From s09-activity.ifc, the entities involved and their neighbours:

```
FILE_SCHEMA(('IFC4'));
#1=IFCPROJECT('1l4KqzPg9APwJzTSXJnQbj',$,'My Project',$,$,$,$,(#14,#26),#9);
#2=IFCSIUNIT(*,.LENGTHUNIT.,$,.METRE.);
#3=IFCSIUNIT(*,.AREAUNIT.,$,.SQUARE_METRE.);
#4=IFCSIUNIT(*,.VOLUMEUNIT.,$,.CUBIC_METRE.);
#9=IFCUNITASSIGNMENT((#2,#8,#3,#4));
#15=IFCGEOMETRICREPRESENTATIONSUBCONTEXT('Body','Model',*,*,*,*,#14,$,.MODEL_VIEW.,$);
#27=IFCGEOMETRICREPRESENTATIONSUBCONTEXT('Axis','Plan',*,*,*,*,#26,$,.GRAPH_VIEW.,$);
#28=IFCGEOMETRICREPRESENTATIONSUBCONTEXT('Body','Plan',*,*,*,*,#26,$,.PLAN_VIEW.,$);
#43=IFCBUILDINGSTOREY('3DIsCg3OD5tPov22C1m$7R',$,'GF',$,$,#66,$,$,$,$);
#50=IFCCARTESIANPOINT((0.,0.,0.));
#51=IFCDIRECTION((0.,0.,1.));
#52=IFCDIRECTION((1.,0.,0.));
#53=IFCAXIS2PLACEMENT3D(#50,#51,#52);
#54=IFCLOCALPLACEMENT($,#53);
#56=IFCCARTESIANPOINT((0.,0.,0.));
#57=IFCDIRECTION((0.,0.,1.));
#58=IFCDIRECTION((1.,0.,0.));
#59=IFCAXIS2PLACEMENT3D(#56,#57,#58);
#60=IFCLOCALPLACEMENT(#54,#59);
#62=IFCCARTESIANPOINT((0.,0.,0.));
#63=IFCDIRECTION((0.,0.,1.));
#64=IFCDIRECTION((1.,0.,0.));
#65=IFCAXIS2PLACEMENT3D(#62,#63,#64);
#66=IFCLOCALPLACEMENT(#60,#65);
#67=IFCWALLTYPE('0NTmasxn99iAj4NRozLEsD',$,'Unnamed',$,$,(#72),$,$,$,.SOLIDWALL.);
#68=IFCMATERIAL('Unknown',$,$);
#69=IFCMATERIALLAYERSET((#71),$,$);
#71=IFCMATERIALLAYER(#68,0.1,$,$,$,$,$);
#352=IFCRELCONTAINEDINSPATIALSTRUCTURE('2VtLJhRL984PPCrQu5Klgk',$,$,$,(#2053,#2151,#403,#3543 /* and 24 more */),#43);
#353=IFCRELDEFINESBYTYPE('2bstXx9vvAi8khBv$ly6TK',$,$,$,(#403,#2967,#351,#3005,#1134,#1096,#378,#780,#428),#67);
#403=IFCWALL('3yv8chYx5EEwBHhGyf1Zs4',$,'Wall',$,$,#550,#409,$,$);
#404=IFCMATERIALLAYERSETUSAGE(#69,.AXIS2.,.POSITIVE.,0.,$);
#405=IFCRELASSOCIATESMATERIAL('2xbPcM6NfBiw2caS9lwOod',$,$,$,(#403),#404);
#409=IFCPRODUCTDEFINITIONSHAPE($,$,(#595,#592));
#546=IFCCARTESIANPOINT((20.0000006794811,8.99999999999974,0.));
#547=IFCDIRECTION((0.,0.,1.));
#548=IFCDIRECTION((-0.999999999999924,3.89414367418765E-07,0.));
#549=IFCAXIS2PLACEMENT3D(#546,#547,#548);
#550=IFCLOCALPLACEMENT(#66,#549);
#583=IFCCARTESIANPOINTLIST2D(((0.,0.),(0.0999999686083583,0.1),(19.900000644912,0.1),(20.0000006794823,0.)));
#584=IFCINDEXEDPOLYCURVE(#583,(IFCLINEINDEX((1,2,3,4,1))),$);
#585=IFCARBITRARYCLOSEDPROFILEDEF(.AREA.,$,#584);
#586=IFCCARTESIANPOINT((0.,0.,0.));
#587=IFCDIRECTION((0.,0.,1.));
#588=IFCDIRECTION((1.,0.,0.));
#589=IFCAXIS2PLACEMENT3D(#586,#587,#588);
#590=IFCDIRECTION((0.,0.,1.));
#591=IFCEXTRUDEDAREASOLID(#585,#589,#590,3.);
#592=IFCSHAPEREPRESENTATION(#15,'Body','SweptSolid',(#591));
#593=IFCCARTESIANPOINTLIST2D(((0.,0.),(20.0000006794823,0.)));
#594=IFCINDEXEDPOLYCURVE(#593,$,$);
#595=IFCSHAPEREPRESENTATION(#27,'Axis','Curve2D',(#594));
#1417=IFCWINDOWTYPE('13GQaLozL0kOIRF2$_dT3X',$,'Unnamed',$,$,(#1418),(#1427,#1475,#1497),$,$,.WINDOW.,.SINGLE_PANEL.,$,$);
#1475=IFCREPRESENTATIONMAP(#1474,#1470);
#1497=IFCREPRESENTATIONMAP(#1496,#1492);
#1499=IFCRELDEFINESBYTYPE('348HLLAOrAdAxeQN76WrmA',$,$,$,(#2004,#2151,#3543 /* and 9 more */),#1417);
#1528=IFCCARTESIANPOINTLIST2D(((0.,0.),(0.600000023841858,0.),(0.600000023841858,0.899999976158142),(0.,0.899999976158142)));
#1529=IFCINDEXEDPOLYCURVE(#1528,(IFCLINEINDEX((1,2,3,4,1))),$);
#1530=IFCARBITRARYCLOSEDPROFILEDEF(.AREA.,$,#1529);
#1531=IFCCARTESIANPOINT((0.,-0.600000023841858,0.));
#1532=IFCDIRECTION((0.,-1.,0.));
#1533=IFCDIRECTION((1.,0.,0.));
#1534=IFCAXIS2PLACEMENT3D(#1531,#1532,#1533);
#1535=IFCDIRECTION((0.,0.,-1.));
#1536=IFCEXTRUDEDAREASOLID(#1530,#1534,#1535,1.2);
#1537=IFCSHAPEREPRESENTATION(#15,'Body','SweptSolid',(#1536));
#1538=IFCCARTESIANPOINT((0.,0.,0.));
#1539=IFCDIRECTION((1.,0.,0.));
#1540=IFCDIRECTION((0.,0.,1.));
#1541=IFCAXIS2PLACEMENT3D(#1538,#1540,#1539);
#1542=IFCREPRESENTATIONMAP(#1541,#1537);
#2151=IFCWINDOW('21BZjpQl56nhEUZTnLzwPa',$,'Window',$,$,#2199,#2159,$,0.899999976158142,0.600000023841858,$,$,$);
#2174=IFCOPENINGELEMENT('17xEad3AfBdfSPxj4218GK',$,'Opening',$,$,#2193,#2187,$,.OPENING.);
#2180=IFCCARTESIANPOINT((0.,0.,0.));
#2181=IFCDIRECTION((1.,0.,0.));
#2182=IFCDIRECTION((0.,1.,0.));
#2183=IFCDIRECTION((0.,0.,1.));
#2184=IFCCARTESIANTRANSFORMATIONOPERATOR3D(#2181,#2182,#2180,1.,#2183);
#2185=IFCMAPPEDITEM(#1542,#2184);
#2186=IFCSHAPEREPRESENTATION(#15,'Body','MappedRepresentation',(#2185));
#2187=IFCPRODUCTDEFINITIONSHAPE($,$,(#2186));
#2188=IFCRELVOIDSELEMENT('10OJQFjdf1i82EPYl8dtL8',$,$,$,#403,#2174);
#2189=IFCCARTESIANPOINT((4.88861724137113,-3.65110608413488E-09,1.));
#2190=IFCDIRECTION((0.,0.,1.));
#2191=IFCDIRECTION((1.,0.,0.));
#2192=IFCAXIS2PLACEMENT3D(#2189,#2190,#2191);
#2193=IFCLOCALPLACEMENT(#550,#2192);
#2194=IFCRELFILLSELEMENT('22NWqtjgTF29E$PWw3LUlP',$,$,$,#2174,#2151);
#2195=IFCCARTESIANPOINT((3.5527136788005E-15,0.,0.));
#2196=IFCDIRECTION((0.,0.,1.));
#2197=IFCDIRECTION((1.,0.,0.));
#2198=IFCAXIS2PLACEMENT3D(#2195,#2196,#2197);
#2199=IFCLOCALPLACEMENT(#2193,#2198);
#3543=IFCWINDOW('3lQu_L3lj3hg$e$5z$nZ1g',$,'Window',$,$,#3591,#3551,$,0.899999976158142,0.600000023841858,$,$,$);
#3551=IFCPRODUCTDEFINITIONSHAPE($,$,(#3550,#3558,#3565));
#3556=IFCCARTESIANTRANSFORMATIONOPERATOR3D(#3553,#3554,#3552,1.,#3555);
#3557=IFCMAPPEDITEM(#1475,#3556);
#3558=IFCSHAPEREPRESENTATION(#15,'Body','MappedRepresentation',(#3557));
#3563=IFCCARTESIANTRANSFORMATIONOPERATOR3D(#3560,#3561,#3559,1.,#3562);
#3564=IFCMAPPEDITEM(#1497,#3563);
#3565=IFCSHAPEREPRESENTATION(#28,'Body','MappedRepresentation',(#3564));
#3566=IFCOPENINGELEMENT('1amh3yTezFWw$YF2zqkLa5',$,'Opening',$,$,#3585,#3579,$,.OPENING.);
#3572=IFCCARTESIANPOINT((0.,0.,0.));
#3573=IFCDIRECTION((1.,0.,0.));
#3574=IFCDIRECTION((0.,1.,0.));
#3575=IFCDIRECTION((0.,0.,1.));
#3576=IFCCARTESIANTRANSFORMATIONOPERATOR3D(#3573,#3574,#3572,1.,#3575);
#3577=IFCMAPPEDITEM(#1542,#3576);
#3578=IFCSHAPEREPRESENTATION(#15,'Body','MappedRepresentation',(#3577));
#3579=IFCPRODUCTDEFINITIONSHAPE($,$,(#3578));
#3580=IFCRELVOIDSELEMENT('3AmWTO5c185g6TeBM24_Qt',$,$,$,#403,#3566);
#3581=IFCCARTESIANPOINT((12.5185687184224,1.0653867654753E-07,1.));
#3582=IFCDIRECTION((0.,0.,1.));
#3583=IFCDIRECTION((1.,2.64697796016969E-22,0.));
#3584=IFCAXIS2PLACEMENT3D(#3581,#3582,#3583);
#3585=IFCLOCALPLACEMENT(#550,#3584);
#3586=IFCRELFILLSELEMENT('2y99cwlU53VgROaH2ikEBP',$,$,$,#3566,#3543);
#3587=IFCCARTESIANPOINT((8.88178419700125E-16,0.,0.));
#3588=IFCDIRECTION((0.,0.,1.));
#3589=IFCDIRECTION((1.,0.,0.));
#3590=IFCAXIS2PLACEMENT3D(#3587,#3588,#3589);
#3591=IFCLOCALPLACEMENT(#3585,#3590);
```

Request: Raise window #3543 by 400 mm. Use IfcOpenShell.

```python
import numpy as np
import ifcopenshell
import ifcopenshell.api.geometry
import ifcopenshell.util.placement
import ifcopenshell.util.unit

model = ifcopenshell.open("s09-activity.ifc")
unit_scale = ifcopenshell.util.unit.calculate_unit_scale(model)

window = model.by_id(3543)
opening = window.FillsVoids[0].RelatingOpeningElement
dz = 0.4 / unit_scale

shift = np.array([0.0, 0.0, dz])
# The window is placed relative to its opening, so it follows when the opening moves.
matrix = ifcopenshell.util.placement.get_local_placement(opening.ObjectPlacement)
matrix[:3, 3] += shift
ifcopenshell.api.geometry.edit_object_placement(
    model, product=opening, matrix=matrix, is_si=False, should_transform_children=True
)

print(f"moved by {dz * unit_scale:+.3f} m")

model.write("s09-activity_v2.ifc")
```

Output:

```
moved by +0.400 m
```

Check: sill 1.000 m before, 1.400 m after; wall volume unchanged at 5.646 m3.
